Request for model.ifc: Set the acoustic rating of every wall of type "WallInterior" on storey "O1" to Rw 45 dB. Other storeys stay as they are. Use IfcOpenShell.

First a look at what the model holds.

```python
import ifcopenshell
import ifcopenshell.util.element

model = ifcopenshell.open("model.ifc")
print(model.schema)
storey = next(s for s in model.by_type("IfcBuildingStorey") if s.Name == "O1")
walls = [e for e in ifcopenshell.util.element.get_decomposition(storey) if e.is_a("IfcWall")]
seen = {}
for e in walls:
    element_type = ifcopenshell.util.element.get_type(e)
    key = (element_type.Name if element_type != e and element_type else None, ifcopenshell.util.element.get_pset(e, "Pset_WallCommon", "AcousticRating"))
    seen[key] = seen.get(key, 0) + 1
for (name, value), count in sorted(seen.items(), key=str):
    print(count, "x", name, "|", value)
```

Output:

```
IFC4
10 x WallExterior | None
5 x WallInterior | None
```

```python
import ifcopenshell
import ifcopenshell.api.pset
import ifcopenshell.util.element

model = ifcopenshell.open("model.ifc")

storey = next(s for s in model.by_type("IfcBuildingStorey") if s.Name == "O1")
walls = [e for e in ifcopenshell.util.element.get_decomposition(storey) if e.is_a("IfcWall")]

count = 0
for e in walls:
    element_type = ifcopenshell.util.element.get_type(e)
    if element_type in (None, e) or element_type.Name != "WallInterior":
        continue
    # add_pset returns the element's existing set when there is one.
    pset = ifcopenshell.api.pset.add_pset(model, product=e, name="Pset_WallCommon")
    ifcopenshell.api.pset.edit_pset(model, pset=pset, properties={"AcousticRating": "Rw 45 dB"})
    count += 1

print(count, "walls updated")

model.write("model_rev.ifc")
```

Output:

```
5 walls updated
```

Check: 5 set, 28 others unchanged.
